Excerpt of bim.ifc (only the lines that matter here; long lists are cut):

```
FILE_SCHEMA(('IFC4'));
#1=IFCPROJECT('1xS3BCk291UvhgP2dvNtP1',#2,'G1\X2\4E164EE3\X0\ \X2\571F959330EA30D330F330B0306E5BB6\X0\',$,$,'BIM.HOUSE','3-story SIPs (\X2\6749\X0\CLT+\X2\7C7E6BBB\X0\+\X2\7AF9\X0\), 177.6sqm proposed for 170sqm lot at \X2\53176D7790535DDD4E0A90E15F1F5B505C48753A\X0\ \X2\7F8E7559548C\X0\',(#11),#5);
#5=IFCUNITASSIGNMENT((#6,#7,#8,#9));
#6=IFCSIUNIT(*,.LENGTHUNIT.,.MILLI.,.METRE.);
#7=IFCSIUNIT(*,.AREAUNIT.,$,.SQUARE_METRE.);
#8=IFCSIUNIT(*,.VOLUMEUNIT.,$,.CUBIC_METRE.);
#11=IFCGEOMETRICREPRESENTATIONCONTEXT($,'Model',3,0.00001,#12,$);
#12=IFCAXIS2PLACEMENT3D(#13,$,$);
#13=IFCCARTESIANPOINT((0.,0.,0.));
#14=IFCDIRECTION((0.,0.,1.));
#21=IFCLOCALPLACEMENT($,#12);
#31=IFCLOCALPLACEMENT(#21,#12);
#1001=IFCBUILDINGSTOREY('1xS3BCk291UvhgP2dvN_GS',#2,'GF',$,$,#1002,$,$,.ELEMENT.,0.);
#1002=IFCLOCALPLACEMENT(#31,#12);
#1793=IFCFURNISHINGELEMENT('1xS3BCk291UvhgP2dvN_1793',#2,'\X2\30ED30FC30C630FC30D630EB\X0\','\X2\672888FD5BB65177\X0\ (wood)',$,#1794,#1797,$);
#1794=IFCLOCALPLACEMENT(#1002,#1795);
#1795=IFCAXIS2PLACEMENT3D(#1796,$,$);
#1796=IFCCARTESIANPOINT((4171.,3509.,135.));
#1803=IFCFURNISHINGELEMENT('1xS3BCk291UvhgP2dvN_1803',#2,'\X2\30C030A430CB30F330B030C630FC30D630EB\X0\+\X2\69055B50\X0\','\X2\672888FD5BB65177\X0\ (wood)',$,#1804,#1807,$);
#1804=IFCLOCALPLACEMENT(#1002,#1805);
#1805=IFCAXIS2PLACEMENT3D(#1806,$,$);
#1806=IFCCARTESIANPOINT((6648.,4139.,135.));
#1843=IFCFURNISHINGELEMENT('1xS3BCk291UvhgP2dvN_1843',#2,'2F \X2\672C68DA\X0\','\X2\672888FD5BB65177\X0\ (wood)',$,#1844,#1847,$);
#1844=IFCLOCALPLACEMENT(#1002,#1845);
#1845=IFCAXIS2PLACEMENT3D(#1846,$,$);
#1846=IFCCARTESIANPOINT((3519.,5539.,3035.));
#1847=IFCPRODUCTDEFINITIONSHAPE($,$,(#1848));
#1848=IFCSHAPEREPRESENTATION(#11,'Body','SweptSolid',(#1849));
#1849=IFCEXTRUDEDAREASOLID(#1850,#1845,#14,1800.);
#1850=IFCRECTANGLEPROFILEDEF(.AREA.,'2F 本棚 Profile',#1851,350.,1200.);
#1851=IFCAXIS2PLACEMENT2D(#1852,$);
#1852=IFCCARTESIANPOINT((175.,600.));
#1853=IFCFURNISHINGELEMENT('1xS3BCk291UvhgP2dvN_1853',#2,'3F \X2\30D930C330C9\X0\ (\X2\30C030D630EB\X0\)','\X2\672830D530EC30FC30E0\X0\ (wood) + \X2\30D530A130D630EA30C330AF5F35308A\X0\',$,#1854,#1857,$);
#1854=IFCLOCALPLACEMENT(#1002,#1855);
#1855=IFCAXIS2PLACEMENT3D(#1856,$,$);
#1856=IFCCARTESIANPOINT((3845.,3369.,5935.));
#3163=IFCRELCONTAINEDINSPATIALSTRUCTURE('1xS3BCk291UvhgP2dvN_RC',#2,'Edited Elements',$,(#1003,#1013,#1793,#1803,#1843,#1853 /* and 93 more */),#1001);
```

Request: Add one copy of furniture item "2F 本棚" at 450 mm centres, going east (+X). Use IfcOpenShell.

```python
import numpy as np
import ifcopenshell
import ifcopenshell.api.geometry
import ifcopenshell.api.root
import ifcopenshell.util.element
import ifcopenshell.util.placement

model = ifcopenshell.open("bim.ifc")


def reuse_history(source, copy):
    """copy_class also copies each property set's owner history, people and application; keep the originals."""
    for rel in copy.IsDefinedBy:
        if rel.is_a("IfcRelDefinesByProperties") and (history := rel.RelatingPropertyDefinition.OwnerHistory):
            rel.RelatingPropertyDefinition.OwnerHistory = source.OwnerHistory
            ifcopenshell.util.element.remove_deep2(model, history)


source = model.by_id(1843)
base = ifcopenshell.util.placement.get_local_placement(source.ObjectPlacement)
step = np.array([1.0, 0.0, 0.0]) * 450.0

for i in range(1, 2):
    copy = ifcopenshell.api.root.copy_class(model, product=source)
    copy.Representation = ifcopenshell.util.element.copy_deep(
        model, source.Representation, exclude=["IfcGeometricRepresentationContext", "IfcRepresentationMap"]
    )
    reuse_history(source, copy)
    matrix = base.copy()
    matrix[:3, 3] += i * step
    print("added at", matrix[:3, 3].round(3) + 0.0)
    ifcopenshell.api.geometry.edit_object_placement(model, product=copy, matrix=matrix, is_si=False)

model.write("bim_v2.ifc")
```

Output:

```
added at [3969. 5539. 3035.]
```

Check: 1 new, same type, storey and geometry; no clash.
